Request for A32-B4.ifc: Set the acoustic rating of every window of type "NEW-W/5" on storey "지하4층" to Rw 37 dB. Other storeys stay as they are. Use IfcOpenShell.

First a look at what the model holds.

```python
import ifcopenshell
import ifcopenshell.util.element

model = ifcopenshell.open("A32-B4.ifc")
print(model.schema)
storey = next(s for s in model.by_type("IfcBuildingStorey") if s.Name == "지하4층")
windows = [e for e in ifcopenshell.util.element.get_decomposition(storey) if e.is_a("IfcWindow")]
seen = {}
for e in windows:
    element_type = ifcopenshell.util.element.get_type(e)
    key = (element_type.Name if element_type != e and element_type else None, ifcopenshell.util.element.get_pset(e, "Pset_WindowCommon", "AcousticRating"))
    seen[key] = seen.get(key, 0) + 1
for (name, value), count in sorted(seen.items(), key=str):
    print(count, "x", name, "|", value)
```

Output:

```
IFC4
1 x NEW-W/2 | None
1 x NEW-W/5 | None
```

```python
import ifcopenshell
import ifcopenshell.api.pset
import ifcopenshell.util.element

model = ifcopenshell.open("A32-B4.ifc")

storey = next(s for s in model.by_type("IfcBuildingStorey") if s.Name == "지하4층")
windows = [e for e in ifcopenshell.util.element.get_decomposition(storey) if e.is_a("IfcWindow")]

count = 0
for e in windows:
    element_type = ifcopenshell.util.element.get_type(e)
    if element_type in (None, e) or element_type.Name != "NEW-W/5":
        continue
    # add_pset returns the element's existing set when there is one.
    pset = ifcopenshell.api.pset.add_pset(model, product=e, name="Pset_WindowCommon")
    ifcopenshell.api.pset.edit_pset(model, pset=pset, properties={"AcousticRating": "Rw 37 dB"})
    count += 1

print(count, "windows updated")

model.write("A32-B4_updated.ifc")
```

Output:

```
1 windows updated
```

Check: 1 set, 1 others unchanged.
